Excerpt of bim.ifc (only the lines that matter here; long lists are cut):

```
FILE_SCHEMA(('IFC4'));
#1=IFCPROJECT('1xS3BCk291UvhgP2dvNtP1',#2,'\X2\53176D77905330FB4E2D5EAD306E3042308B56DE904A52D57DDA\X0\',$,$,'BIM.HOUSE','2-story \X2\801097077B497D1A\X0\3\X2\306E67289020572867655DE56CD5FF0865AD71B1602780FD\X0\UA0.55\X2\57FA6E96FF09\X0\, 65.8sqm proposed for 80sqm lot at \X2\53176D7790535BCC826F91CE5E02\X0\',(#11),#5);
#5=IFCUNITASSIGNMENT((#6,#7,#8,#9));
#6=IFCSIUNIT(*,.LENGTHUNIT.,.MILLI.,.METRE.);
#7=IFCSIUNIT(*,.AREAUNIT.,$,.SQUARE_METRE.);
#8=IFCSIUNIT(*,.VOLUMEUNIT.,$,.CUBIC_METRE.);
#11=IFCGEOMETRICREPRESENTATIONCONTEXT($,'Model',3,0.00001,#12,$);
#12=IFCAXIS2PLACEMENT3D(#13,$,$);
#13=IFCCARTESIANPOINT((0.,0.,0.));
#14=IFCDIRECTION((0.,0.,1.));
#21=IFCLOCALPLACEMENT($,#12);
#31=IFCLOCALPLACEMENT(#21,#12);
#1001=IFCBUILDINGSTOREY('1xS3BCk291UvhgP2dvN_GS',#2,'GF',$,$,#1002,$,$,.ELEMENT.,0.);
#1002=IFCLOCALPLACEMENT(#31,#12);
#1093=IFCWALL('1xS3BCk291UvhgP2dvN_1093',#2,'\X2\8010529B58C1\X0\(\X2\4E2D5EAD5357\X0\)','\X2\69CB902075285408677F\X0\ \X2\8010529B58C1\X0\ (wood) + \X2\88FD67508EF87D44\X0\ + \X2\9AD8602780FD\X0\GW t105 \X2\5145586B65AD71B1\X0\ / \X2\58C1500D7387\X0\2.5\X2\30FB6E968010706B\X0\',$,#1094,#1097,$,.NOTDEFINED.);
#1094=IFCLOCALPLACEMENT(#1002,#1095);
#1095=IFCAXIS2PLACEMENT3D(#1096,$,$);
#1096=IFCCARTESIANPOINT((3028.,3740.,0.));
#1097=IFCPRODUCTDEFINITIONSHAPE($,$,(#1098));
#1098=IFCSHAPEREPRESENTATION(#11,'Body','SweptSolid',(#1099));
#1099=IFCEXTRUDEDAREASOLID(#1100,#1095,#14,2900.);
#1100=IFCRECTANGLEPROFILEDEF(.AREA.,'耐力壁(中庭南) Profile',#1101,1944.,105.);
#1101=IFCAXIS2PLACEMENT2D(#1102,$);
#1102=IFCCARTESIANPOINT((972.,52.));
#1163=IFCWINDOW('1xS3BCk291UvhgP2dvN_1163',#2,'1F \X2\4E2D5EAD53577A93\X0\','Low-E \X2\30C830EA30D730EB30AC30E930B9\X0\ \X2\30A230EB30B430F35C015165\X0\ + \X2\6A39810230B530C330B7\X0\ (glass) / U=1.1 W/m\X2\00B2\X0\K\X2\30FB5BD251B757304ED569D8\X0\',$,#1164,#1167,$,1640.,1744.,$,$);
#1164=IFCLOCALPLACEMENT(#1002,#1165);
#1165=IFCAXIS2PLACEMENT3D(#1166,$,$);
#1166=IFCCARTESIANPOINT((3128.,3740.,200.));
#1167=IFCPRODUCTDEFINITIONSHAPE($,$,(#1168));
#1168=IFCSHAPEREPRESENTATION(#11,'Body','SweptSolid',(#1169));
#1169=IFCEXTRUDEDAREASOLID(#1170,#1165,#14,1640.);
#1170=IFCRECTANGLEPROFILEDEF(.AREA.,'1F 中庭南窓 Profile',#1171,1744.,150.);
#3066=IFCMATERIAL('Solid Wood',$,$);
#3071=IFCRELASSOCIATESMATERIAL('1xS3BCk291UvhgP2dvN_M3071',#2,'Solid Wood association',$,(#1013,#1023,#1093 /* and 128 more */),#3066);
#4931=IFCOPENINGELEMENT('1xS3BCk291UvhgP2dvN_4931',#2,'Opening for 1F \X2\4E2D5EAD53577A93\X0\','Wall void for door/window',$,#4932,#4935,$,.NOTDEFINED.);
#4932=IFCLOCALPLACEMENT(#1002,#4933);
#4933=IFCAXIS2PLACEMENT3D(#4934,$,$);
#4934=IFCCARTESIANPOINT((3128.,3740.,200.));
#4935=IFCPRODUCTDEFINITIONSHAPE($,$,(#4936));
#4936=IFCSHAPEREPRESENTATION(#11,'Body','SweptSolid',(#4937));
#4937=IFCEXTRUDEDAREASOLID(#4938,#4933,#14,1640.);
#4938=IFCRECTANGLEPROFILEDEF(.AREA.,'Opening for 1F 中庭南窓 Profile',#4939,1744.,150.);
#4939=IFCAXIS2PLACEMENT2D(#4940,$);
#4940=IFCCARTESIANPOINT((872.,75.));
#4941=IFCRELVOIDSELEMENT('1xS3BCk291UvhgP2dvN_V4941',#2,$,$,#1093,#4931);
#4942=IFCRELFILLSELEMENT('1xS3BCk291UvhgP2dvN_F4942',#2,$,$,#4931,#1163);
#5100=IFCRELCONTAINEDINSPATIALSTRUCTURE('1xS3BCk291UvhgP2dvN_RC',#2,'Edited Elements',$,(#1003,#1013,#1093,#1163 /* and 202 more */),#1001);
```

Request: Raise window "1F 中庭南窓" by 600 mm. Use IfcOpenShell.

```python
import numpy as np
import ifcopenshell
import ifcopenshell.api.geometry
import ifcopenshell.util.placement
import ifcopenshell.util.unit

model = ifcopenshell.open("bim.ifc")
unit_scale = ifcopenshell.util.unit.calculate_unit_scale(model)

window = model.by_guid("1xS3BCk291UvhgP2dvN_1163")
opening = window.FillsVoids[0].RelatingOpeningElement
dz = 0.6 / unit_scale

shift = np.array([0.0, 0.0, dz])
# The window is not placed relative to its opening, so move both.
for product in (opening, window):
    matrix = ifcopenshell.util.placement.get_local_placement(product.ObjectPlacement)
    matrix[:3, 3] += shift
    ifcopenshell.api.geometry.edit_object_placement(model, product=product, matrix=matrix, is_si=False)

print(f"moved by {dz * unit_scale:+.3f} m")

model.write("bim_rev.ifc")
```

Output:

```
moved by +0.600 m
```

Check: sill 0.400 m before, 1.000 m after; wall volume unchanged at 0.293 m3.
